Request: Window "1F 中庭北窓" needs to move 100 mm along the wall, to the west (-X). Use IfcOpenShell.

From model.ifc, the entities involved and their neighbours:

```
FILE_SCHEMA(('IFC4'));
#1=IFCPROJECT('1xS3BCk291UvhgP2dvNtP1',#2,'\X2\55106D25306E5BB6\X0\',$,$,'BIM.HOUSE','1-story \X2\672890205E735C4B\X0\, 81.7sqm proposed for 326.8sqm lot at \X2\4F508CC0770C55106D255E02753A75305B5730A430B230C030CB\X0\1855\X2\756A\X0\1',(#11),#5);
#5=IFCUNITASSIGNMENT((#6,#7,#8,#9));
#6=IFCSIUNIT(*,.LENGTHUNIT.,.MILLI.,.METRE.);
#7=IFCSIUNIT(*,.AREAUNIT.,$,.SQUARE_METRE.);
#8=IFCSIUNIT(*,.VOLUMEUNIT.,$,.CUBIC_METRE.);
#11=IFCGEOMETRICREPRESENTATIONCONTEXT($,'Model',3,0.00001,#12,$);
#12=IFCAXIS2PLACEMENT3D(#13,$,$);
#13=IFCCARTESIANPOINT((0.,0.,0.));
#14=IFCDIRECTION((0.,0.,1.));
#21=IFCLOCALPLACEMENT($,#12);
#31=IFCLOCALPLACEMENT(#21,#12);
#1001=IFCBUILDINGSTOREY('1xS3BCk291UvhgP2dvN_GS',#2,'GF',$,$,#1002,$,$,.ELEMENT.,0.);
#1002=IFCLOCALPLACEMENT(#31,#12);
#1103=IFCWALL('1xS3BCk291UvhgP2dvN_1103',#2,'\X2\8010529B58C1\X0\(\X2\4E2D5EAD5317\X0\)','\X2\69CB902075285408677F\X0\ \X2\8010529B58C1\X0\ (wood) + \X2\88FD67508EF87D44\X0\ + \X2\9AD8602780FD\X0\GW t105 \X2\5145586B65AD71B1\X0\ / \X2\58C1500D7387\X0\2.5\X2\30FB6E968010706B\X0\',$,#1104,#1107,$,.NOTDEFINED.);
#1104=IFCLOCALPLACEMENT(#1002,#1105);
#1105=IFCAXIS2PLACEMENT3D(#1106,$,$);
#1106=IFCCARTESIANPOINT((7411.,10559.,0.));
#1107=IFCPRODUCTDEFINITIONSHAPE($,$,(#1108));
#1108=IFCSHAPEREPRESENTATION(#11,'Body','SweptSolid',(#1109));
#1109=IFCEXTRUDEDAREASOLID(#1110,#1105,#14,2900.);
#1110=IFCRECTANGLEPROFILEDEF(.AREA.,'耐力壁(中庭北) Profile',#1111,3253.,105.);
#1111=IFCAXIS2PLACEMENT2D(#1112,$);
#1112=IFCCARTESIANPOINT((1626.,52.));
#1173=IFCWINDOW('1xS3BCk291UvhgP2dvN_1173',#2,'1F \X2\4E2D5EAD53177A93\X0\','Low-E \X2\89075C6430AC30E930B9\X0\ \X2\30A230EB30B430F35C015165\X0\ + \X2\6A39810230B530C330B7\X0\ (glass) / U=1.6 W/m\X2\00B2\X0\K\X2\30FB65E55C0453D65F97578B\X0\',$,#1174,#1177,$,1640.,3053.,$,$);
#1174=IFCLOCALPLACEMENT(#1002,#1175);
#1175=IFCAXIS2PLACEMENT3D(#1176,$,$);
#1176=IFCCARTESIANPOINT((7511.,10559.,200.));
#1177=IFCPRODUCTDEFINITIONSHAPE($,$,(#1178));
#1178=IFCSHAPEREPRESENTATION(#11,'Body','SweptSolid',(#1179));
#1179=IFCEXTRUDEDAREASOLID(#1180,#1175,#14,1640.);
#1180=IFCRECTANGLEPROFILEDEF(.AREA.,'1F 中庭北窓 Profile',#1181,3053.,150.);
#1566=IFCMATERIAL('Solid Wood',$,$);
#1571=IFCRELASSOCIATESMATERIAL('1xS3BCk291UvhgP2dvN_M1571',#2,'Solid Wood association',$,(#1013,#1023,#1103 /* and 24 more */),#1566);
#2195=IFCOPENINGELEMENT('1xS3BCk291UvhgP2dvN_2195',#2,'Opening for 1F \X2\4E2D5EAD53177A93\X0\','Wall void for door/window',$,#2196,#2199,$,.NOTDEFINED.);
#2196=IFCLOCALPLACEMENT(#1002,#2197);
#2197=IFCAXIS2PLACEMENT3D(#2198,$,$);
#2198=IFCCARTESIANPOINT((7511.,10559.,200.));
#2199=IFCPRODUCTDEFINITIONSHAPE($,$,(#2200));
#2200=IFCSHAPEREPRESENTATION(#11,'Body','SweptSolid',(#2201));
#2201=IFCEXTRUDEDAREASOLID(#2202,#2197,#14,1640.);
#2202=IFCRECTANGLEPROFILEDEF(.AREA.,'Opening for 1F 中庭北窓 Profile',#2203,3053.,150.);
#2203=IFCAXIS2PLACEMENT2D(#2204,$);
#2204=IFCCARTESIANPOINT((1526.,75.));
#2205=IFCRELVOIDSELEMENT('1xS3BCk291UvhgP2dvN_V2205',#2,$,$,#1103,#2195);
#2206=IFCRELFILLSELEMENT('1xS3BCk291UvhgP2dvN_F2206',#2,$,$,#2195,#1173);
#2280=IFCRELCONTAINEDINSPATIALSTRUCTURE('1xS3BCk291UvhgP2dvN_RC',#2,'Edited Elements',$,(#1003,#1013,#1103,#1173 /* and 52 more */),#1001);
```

```python
import ifcopenshell
import ifcopenshell.api.geometry
import ifcopenshell.util.placement
import ifcopenshell.util.unit

model = ifcopenshell.open("model.ifc")
unit_scale = ifcopenshell.util.unit.calculate_unit_scale(model)

window = model.by_guid("1xS3BCk291UvhgP2dvN_1173")
opening = window.FillsVoids[0].RelatingOpeningElement
wall = opening.VoidsElements[0].RelatingBuildingElement

wall_matrix = ifcopenshell.util.placement.get_local_placement(wall.ObjectPlacement)
shift = wall_matrix[:3, 0] * -0.1 / unit_scale
before = ifcopenshell.util.placement.get_local_placement(window.ObjectPlacement)[:3, 3].copy()

# The window is not placed relative to its opening, so move both.
for product in (opening, window):
    matrix = ifcopenshell.util.placement.get_local_placement(product.ObjectPlacement)
    matrix[:3, 3] += shift
    ifcopenshell.api.geometry.edit_object_placement(model, product=product, matrix=matrix, is_si=False)

after = ifcopenshell.util.placement.get_local_placement(window.ObjectPlacement)[:3, 3]
print("window moved by", (after - before).round(3) + 0.0)

model.write("model_rev.ifc")
```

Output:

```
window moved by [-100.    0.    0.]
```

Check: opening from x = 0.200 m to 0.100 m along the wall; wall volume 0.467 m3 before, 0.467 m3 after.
